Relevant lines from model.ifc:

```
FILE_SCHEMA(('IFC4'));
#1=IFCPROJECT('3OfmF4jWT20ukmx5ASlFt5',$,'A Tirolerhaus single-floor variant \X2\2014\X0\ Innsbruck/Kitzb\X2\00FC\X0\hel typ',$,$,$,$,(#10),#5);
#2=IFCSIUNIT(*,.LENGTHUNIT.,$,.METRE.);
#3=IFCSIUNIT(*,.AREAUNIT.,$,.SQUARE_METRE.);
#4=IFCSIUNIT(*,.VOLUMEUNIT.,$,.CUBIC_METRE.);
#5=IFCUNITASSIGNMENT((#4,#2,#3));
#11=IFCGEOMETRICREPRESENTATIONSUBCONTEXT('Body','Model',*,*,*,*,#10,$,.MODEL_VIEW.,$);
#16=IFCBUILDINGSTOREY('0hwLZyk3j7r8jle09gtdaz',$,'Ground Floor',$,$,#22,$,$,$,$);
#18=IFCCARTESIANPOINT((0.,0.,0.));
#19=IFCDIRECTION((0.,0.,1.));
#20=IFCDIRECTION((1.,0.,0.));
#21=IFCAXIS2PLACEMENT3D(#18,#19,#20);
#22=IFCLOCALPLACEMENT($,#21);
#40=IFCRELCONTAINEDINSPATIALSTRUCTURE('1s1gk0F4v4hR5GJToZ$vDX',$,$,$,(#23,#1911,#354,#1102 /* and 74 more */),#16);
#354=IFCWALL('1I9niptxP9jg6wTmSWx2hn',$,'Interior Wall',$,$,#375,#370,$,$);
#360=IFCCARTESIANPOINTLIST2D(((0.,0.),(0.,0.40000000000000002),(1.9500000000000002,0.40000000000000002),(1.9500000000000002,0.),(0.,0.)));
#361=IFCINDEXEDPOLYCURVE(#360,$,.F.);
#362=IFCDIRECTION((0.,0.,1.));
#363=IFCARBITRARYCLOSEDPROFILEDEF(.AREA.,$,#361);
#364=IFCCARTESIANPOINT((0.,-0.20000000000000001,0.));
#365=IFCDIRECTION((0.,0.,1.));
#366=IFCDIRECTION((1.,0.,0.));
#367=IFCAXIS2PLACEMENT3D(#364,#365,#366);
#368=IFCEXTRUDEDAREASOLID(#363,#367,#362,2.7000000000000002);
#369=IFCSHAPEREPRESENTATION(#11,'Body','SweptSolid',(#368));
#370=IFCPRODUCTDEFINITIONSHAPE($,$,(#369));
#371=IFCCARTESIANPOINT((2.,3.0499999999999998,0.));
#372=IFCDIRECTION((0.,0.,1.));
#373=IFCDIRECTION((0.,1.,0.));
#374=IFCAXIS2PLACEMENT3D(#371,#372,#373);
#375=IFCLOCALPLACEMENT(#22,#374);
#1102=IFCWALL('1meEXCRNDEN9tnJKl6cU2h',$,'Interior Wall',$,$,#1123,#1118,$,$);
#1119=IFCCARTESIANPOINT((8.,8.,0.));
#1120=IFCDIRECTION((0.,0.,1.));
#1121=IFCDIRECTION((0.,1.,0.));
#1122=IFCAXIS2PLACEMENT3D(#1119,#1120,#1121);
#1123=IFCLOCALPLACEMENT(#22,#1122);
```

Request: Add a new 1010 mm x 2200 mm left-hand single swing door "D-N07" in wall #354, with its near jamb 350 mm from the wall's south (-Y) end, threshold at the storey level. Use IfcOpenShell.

```python
import numpy as np
import ifcopenshell
import ifcopenshell.api.feature
import ifcopenshell.api.geometry
import ifcopenshell.api.root
import ifcopenshell.api.spatial
import ifcopenshell.geom
import ifcopenshell.util.element
import ifcopenshell.util.placement
import ifcopenshell.util.representation
import ifcopenshell.util.shape
import ifcopenshell.util.unit

model = ifcopenshell.open("model.ifc")
unit_scale = ifcopenshell.util.unit.calculate_unit_scale(model)
settings = ifcopenshell.geom.settings()


def volume(element):
    """Net volume in cubic metres, openings subtracted."""
    shape = ifcopenshell.geom.create_shape(settings, element)
    return ifcopenshell.util.shape.get_volume(shape.geometry)


wall = model.by_guid("1I9niptxP9jg6wTmSWx2hn")
storey = ifcopenshell.util.element.get_container(wall, ifc_class="IfcBuildingStorey")
context = ifcopenshell.util.representation.get_context(model, "Model", "Body", "MODEL_VIEW")
before = volume(wall)

width, height, from_end, sill = 1.01, 2.2, 0.35, 0.0  # metres

# The wall runs along its own X axis, and the end named is its -X end.
wall_shape = ifcopenshell.geom.create_shape(settings, wall)
x, y, z = ifcopenshell.util.shape.get_vertices(wall_shape.geometry).T
start = x.min() + from_end
face, thickness = float(y.min()), float(y.max() - y.min())
wall_matrix = ifcopenshell.util.placement.get_local_placement(wall.ObjectPlacement)
level = ifcopenshell.util.placement.get_local_placement(storey.ObjectPlacement)[2, 3]


def in_wall(x, y):
    """Placement at x, y metres in the wall's axes, at sill height."""
    matrix = wall_matrix.copy()
    matrix[:, 3] = wall_matrix @ np.array([x / unit_scale, y / unit_scale, 0.0, 1.0])
    matrix[2, 3] = level + sill / unit_scale
    return matrix


# Opening: a box that overshoots both wall faces by 50 mm.
opening = ifcopenshell.api.root.create_entity(model, ifc_class="IfcOpeningElement", predefined_type="OPENING")
box = ifcopenshell.api.geometry.add_wall_representation(
    model, context=context, length=width, height=height, thickness=thickness + 0.1
)
ifcopenshell.api.geometry.assign_representation(model, product=opening, representation=box)
ifcopenshell.api.geometry.edit_object_placement(model, product=opening, matrix=in_wall(start, face - 0.05), is_si=False)
ifcopenshell.api.feature.add_feature(model, feature=opening, element=wall)

door = ifcopenshell.api.root.create_entity(model, ifc_class="IfcDoor", name="D-N07", predefined_type="DOOR")
door.OverallWidth, door.OverallHeight = width / unit_scale, height / unit_scale
door.OperationType = "SINGLE_SWING_LEFT"
body = ifcopenshell.api.geometry.add_door_representation(
    model,
    context=context,
    overall_width=door.OverallWidth,
    overall_height=door.OverallHeight,
    operation_type="SINGLE_SWING_LEFT",
    lining_properties={"LiningDepth": thickness / unit_scale, "ThresholdDepth": thickness / unit_scale},
)
ifcopenshell.api.geometry.assign_representation(model, product=door, representation=body)
ifcopenshell.api.spatial.assign_container(model, products=[door], relating_structure=storey)
ifcopenshell.api.feature.add_filling(model, opening=opening, element=door)

# The lining spans the wall, so the door starts at the wall face.
ifcopenshell.api.geometry.edit_object_placement(model, product=door, matrix=in_wall(start, face), is_si=False)

after = volume(wall)

print(f"wall volume {before:.3f} -> {after:.3f} m3")

model.write("model_updated.ifc")
```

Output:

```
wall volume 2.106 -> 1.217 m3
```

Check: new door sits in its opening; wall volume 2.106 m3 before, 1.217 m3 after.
